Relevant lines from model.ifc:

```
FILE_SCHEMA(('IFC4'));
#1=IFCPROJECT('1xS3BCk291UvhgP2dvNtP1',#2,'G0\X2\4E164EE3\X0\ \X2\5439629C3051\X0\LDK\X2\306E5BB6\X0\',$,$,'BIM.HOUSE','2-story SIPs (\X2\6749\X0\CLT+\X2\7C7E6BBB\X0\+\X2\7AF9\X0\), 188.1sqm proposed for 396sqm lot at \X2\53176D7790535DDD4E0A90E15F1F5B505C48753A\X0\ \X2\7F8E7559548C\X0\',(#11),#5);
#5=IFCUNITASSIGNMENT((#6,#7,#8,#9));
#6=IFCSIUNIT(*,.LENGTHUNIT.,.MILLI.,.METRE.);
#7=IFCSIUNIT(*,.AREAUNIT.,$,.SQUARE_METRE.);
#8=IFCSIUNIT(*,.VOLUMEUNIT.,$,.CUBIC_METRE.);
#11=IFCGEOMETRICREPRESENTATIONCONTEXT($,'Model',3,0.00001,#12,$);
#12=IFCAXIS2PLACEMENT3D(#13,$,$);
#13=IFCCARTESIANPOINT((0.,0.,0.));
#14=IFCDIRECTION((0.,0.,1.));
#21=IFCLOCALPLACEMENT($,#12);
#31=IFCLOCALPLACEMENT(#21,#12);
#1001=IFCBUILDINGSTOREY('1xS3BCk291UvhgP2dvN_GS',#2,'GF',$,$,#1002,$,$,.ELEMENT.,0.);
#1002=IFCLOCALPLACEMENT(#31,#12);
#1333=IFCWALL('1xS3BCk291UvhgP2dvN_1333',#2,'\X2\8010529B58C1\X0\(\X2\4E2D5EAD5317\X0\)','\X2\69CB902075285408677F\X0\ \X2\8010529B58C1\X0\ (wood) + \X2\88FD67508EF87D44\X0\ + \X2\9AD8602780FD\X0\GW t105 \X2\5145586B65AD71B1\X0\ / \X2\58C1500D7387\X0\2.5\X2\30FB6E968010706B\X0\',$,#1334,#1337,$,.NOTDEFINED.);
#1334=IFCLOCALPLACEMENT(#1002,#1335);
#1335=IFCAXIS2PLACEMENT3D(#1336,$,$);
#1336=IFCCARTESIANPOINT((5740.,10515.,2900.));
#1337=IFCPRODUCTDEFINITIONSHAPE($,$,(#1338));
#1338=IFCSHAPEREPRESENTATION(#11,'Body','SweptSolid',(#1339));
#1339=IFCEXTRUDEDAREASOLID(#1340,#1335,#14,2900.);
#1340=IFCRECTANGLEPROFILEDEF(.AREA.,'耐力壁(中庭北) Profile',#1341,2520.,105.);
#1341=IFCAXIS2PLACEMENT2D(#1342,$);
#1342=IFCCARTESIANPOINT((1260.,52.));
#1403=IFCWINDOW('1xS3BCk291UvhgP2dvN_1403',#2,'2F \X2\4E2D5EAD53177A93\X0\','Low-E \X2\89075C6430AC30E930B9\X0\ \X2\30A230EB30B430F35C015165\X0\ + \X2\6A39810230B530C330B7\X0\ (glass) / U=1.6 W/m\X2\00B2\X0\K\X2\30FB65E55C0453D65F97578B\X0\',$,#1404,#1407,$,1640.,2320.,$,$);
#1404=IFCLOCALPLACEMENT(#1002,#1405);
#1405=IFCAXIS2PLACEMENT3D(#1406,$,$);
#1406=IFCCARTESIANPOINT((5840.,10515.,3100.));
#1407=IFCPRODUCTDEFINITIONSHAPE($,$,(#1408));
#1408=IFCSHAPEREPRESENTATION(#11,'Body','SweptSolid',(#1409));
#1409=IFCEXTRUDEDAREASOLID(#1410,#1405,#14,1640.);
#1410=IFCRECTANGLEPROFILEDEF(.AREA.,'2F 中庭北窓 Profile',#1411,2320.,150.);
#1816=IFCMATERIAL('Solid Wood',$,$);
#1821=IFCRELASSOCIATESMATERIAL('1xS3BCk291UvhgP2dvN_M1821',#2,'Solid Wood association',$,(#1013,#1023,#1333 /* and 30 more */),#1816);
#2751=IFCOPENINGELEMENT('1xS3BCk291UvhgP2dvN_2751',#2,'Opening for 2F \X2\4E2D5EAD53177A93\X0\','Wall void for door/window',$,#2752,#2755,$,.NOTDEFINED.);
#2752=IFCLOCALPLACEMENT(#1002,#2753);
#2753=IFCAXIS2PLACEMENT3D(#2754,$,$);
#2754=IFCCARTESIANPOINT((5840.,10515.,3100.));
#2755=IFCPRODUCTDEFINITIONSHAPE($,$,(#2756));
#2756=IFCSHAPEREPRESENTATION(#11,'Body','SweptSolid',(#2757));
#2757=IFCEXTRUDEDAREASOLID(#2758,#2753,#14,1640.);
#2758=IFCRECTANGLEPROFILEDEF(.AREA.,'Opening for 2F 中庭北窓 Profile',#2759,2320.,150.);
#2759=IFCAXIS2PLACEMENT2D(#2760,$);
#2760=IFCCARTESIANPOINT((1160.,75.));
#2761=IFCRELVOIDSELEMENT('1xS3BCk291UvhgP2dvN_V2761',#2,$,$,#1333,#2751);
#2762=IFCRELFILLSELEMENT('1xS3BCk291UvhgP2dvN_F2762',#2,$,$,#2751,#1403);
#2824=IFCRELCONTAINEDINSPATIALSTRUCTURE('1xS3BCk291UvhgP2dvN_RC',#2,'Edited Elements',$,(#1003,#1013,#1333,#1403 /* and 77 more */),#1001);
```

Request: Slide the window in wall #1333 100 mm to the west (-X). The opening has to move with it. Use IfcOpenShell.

```python
import ifcopenshell
import ifcopenshell.api.geometry
import ifcopenshell.util.placement

model = ifcopenshell.open("model.ifc")

window = model.by_id(1403)
opening = window.FillsVoids[0].RelatingOpeningElement
wall = opening.VoidsElements[0].RelatingBuildingElement

wall_matrix = ifcopenshell.util.placement.get_local_placement(wall.ObjectPlacement)
shift = wall_matrix[:3, 0] * -100.0
before = ifcopenshell.util.placement.get_local_placement(window.ObjectPlacement)[:3, 3].copy()

# The window is not placed relative to its opening, so move both.
for product in (opening, window):
    matrix = ifcopenshell.util.placement.get_local_placement(product.ObjectPlacement)
    matrix[:3, 3] += shift
    ifcopenshell.api.geometry.edit_object_placement(model, product=product, matrix=matrix, is_si=False)

after = ifcopenshell.util.placement.get_local_placement(window.ObjectPlacement)[:3, 3]
print("window moved by", (after - before).round(3) + 0.0)

model.write("model_edited.ifc")
```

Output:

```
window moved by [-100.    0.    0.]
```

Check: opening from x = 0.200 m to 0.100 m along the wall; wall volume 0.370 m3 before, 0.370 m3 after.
